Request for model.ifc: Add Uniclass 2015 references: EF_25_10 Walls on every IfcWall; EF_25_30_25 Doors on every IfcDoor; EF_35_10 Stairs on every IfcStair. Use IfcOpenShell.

First a look at what the model holds.

```python
import ifcopenshell

model = ifcopenshell.open("model.ifc")
print(model.schema)
print("classifications:", [c.Name for c in model.by_type("IfcClassification")])
for ifc_class in ("IfcDoor", "IfcRoof", "IfcStair", "IfcWall", "IfcWindow"):
    print(ifc_class, len(model.by_type(ifc_class)))
```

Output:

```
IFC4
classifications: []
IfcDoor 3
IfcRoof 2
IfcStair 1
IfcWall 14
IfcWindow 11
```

```python
import ifcopenshell
import ifcopenshell.api.classification

model = ifcopenshell.open("model.ifc")

system = ifcopenshell.api.classification.add_classification(model, classification="Uniclass 2015")

codes = {
    "IfcWall": ("EF_25_10", "Walls"),
    "IfcDoor": ("EF_25_30_25", "Doors"),
    "IfcStair": ("EF_35_10", "Stairs"),
}
for ifc_class, (code, name) in codes.items():
    products = model.by_type(ifc_class)
    ifcopenshell.api.classification.add_reference(
        model, products=products, classification=system, identification=code, name=name
    )
    print(code, len(products))

model.write("model_updated.ifc")
```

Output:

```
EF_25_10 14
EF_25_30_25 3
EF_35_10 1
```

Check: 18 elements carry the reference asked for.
